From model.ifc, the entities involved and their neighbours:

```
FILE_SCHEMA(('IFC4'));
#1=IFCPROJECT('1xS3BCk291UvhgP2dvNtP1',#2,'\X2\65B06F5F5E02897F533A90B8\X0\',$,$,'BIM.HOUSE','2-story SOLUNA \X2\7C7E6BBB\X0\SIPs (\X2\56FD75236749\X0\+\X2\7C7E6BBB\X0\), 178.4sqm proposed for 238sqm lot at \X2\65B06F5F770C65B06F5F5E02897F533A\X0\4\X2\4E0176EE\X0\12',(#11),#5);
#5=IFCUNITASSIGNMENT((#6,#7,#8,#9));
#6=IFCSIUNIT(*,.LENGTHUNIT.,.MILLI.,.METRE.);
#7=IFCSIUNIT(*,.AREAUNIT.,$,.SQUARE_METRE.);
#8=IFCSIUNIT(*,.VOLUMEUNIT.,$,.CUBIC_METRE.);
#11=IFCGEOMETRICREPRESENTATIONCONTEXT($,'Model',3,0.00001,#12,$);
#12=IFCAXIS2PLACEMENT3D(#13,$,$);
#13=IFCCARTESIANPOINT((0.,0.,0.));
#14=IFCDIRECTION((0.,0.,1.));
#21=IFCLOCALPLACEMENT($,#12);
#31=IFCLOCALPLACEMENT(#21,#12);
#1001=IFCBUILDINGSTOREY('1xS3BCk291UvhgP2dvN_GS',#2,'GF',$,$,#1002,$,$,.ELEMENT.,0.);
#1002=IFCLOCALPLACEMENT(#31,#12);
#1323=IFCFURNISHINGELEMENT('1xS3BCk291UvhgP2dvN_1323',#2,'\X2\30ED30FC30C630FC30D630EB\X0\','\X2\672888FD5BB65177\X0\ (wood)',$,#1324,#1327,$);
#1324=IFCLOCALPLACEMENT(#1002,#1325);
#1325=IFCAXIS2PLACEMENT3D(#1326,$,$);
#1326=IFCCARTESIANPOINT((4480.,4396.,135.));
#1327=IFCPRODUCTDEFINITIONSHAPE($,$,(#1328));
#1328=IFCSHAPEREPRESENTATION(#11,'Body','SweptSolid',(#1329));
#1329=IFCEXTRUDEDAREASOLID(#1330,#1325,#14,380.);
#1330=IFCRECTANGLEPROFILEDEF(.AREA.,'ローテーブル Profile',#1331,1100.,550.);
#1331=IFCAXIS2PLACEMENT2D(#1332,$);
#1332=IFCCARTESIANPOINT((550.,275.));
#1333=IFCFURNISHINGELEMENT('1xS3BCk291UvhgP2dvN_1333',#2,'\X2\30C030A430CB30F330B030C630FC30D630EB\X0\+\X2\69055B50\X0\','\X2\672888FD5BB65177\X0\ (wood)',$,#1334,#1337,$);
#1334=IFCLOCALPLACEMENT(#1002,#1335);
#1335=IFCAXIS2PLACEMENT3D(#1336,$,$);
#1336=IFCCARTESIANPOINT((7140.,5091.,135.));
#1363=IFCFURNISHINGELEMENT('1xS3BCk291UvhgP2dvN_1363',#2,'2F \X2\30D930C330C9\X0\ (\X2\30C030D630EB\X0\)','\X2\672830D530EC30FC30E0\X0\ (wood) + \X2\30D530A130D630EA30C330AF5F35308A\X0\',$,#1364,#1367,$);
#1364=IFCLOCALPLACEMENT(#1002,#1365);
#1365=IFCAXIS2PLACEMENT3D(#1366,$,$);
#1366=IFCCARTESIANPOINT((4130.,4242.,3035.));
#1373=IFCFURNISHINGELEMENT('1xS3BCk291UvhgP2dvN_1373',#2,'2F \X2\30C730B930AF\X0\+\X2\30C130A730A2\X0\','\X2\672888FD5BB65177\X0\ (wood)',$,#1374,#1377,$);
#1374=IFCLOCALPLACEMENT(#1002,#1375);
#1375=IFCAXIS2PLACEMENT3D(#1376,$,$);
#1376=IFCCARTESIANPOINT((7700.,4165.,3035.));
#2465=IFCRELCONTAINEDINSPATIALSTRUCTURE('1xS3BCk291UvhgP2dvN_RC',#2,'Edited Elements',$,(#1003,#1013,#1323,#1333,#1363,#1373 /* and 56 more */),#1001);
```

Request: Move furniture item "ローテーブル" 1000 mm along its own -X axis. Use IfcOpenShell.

```python
import ifcopenshell
import ifcopenshell.api.geometry
import ifcopenshell.util.placement
import ifcopenshell.util.unit

model = ifcopenshell.open("model.ifc")
unit_scale = ifcopenshell.util.unit.calculate_unit_scale(model)

item = model.by_guid("1xS3BCk291UvhgP2dvN_1323")
matrix = ifcopenshell.util.placement.get_local_placement(item.ObjectPlacement)
matrix[:3, 3] -= matrix[:3, 0] * 1 / unit_scale
ifcopenshell.api.geometry.edit_object_placement(model, product=item, matrix=matrix, is_si=False)

print(ifcopenshell.util.placement.get_local_placement(item.ObjectPlacement).round(3) + 0.0)

model.write("model-out.ifc")
```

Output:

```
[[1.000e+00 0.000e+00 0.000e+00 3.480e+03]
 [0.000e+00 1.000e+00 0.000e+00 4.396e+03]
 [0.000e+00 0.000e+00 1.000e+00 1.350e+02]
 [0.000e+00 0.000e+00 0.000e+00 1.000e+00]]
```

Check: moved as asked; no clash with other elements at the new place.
